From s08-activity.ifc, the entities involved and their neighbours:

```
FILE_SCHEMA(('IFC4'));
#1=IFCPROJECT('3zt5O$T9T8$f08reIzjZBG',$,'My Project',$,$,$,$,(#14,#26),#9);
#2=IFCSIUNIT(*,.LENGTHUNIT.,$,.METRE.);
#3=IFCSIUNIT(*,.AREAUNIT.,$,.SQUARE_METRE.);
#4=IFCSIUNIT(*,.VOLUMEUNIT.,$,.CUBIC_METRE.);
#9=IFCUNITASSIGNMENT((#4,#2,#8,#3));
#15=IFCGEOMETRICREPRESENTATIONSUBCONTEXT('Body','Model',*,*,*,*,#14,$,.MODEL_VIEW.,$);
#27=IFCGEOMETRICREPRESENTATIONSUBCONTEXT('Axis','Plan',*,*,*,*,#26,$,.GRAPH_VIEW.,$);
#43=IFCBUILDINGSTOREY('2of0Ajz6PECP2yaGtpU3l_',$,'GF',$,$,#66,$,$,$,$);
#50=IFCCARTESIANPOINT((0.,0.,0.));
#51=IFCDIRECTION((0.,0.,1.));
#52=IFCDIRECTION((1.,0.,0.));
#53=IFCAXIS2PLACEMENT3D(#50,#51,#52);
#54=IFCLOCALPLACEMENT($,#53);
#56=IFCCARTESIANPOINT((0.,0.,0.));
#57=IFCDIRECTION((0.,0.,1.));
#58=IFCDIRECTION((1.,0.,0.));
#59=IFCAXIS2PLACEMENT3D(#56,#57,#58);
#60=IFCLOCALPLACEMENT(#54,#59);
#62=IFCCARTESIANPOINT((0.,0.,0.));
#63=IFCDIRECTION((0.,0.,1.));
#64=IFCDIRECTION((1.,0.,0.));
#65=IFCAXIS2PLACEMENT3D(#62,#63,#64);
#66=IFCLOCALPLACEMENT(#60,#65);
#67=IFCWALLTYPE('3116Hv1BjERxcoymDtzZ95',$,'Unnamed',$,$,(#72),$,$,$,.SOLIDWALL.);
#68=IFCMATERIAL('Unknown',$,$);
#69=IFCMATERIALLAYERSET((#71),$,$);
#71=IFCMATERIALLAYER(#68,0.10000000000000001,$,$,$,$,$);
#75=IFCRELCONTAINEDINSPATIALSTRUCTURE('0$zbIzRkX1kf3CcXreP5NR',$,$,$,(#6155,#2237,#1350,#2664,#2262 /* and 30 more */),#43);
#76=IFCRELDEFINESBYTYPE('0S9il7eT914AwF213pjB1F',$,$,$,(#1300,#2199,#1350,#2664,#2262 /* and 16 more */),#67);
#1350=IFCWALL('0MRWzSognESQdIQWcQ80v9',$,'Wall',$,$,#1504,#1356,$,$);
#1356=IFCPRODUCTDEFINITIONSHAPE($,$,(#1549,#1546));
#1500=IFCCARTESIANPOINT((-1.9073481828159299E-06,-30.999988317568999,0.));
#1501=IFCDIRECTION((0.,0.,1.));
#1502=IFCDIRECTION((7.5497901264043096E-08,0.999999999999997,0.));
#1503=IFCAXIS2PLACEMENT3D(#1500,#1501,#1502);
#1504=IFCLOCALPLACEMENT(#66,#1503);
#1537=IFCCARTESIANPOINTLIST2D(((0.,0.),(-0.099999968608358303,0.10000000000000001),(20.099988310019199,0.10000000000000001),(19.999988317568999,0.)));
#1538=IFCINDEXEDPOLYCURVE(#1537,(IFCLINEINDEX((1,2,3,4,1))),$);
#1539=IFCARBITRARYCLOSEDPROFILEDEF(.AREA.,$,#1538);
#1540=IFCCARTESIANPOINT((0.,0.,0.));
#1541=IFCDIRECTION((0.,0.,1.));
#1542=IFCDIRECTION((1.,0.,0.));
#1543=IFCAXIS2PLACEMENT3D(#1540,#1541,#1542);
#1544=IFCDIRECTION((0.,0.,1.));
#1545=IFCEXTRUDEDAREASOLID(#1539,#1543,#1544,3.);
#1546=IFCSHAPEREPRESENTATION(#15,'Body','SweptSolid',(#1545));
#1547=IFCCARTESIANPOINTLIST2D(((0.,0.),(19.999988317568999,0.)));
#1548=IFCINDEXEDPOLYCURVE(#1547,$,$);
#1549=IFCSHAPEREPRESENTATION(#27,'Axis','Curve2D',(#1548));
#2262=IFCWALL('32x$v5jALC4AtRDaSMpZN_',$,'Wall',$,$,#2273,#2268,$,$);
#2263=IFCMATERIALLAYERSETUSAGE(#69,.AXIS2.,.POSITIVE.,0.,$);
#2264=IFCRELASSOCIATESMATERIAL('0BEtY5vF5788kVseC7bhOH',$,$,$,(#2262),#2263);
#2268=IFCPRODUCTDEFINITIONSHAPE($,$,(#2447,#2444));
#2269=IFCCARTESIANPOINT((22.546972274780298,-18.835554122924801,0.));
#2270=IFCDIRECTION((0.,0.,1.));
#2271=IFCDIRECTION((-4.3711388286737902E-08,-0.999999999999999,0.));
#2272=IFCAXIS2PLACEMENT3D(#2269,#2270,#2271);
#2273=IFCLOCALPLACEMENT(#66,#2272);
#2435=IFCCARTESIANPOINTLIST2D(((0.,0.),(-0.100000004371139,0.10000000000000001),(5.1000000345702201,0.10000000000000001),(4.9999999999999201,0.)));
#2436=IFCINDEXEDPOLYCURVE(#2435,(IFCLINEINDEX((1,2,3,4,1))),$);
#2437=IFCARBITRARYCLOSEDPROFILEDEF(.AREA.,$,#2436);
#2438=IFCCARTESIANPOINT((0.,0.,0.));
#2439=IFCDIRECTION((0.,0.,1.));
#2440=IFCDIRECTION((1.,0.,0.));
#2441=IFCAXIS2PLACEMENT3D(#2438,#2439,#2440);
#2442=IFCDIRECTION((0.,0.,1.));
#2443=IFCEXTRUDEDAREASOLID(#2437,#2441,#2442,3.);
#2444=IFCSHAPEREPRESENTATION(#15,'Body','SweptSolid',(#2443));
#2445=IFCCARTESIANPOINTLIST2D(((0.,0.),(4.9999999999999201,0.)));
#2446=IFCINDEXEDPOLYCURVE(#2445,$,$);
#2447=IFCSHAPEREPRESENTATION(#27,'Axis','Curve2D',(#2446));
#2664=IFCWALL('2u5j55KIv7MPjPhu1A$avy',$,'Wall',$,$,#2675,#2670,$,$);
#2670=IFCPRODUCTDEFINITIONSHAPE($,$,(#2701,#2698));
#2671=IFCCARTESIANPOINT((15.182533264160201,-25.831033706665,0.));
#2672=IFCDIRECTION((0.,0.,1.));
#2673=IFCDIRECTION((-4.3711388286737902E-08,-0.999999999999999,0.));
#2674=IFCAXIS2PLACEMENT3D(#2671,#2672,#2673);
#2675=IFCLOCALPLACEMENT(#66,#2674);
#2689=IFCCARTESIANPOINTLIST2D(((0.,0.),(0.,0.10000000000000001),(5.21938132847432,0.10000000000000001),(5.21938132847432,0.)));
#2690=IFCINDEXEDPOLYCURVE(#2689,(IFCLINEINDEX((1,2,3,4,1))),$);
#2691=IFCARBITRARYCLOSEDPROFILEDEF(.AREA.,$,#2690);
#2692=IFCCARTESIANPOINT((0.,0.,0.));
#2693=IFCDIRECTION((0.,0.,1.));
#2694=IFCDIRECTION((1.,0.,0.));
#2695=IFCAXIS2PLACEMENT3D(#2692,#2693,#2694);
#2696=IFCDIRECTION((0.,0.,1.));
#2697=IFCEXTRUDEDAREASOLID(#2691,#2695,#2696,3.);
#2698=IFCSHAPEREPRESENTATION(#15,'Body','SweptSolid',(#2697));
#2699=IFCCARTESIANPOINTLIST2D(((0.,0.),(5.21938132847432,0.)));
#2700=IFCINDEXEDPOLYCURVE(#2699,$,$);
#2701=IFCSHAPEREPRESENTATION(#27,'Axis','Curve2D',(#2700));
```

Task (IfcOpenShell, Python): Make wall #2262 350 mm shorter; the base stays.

```python
import ifcopenshell
import ifcopenshell.geom
import ifcopenshell.util.representation
import ifcopenshell.util.shape
import ifcopenshell.util.unit

model = ifcopenshell.open("s08-activity.ifc")
unit_scale = ifcopenshell.util.unit.calculate_unit_scale(model)
settings = ifcopenshell.geom.settings()


def volume(element):
    """Net volume in cubic metres, openings subtracted."""
    shape = ifcopenshell.geom.create_shape(settings, element)
    return ifcopenshell.util.shape.get_volume(shape.geometry)


wall = model.by_id(2262)
before = volume(wall)

body = ifcopenshell.util.representation.get_representation(wall, "Model", "Body")
solid = body.Items[0]
old_height = solid.Depth
solid.Depth -= 0.35 / unit_scale
after = volume(wall)

print(f"height {old_height:g} -> {solid.Depth:g}, volume {before:.3f} -> {after:.3f} m3")

model.write("s08-activity_updated.ifc")
```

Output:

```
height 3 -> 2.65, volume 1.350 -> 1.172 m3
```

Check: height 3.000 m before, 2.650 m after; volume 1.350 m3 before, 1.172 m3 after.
